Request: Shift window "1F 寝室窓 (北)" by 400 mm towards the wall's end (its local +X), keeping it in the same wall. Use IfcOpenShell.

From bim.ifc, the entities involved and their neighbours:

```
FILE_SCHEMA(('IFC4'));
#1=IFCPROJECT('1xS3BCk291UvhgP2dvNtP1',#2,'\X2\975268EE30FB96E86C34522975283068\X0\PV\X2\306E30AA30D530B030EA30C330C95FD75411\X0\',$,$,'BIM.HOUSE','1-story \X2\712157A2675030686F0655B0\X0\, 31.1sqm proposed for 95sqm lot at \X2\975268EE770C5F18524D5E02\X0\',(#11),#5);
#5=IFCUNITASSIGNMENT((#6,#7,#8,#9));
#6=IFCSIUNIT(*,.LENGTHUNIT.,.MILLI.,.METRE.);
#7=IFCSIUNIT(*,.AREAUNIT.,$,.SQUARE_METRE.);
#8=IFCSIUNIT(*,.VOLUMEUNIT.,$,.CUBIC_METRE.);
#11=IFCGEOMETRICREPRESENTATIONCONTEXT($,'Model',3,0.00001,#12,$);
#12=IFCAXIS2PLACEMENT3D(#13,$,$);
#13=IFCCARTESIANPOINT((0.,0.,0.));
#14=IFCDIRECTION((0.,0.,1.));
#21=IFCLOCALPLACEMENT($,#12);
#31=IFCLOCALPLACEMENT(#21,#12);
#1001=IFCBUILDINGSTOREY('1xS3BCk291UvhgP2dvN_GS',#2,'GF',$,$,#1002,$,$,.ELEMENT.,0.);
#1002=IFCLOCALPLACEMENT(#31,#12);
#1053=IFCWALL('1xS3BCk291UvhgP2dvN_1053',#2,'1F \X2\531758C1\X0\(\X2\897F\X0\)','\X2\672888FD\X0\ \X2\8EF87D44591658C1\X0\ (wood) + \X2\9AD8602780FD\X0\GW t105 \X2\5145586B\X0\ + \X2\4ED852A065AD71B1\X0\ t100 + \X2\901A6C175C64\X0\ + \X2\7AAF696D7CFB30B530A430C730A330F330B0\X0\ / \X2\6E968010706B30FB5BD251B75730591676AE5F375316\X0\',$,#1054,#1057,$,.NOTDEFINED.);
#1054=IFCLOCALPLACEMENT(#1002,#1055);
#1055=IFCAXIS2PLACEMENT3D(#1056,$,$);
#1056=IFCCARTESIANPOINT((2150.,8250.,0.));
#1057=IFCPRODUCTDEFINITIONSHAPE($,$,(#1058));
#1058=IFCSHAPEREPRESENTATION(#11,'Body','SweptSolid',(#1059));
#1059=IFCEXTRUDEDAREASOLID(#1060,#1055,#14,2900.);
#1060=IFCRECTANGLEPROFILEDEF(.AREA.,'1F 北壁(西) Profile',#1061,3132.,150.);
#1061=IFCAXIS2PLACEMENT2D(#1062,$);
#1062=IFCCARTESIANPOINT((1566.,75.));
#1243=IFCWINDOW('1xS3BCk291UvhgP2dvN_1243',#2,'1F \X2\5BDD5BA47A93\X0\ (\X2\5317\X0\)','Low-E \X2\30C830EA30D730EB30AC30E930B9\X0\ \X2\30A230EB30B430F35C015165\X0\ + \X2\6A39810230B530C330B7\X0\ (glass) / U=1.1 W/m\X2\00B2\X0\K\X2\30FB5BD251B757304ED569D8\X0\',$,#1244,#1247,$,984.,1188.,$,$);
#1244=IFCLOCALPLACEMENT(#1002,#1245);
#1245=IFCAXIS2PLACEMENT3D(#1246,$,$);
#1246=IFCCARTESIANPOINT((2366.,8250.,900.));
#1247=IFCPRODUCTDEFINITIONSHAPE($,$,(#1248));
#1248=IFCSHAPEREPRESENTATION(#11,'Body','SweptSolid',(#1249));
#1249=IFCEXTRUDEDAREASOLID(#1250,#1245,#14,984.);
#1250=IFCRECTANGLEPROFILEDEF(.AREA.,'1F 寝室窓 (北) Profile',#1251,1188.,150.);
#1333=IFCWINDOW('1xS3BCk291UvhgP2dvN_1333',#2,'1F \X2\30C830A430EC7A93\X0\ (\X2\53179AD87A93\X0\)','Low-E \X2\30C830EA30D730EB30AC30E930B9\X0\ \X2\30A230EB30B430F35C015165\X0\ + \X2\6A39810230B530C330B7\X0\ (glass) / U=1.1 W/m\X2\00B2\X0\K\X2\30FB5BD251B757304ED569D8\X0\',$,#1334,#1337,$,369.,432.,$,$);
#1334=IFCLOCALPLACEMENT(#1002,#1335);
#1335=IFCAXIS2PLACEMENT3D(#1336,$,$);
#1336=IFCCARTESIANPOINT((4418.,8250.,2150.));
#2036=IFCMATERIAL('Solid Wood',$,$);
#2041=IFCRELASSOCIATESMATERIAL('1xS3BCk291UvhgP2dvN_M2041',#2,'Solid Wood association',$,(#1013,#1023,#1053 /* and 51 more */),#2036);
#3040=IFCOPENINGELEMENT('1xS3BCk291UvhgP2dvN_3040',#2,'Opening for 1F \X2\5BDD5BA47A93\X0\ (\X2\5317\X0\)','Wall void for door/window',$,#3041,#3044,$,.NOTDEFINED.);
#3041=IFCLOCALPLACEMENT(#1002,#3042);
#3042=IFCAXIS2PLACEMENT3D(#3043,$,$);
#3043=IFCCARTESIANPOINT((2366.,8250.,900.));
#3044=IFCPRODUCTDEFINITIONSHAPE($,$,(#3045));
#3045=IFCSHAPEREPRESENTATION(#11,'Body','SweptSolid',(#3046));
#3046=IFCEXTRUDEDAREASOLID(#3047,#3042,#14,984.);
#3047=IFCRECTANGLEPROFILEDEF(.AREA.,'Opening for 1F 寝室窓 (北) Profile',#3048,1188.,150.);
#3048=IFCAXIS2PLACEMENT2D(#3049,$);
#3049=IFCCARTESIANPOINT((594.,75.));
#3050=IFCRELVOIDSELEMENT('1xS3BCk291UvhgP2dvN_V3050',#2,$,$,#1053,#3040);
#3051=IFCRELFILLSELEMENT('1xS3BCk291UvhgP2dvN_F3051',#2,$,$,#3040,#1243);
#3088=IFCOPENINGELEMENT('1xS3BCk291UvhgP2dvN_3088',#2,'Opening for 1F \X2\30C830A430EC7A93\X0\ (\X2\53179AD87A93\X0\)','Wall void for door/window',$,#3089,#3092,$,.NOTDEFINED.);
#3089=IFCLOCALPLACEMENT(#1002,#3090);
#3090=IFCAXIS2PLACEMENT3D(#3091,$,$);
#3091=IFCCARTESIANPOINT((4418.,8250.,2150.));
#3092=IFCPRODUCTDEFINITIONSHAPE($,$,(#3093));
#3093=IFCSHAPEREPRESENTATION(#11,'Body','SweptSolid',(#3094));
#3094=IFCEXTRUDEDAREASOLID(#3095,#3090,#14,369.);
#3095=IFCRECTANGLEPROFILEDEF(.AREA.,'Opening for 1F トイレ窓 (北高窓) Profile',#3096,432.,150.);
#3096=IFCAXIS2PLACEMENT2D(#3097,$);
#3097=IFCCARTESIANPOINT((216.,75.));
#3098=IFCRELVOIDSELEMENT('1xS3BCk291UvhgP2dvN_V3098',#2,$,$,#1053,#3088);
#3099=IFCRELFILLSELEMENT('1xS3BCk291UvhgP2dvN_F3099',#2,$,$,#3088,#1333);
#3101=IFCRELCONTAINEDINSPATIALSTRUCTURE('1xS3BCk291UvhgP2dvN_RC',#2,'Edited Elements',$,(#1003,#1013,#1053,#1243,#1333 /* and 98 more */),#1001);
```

```python
import ifcopenshell
import ifcopenshell.api.geometry
import ifcopenshell.util.placement
import ifcopenshell.util.unit

model = ifcopenshell.open("bim.ifc")
unit_scale = ifcopenshell.util.unit.calculate_unit_scale(model)

window = model.by_guid("1xS3BCk291UvhgP2dvN_1243")
opening = window.FillsVoids[0].RelatingOpeningElement
wall = opening.VoidsElements[0].RelatingBuildingElement

wall_matrix = ifcopenshell.util.placement.get_local_placement(wall.ObjectPlacement)
shift = wall_matrix[:3, 0] * 0.4 / unit_scale
before = ifcopenshell.util.placement.get_local_placement(window.ObjectPlacement)[:3, 3].copy()

# The window is not placed relative to its opening, so move both.
for product in (opening, window):
    matrix = ifcopenshell.util.placement.get_local_placement(product.ObjectPlacement)
    matrix[:3, 3] += shift
    ifcopenshell.api.geometry.edit_object_placement(model, product=product, matrix=matrix, is_si=False)

after = ifcopenshell.util.placement.get_local_placement(window.ObjectPlacement)[:3, 3]
print("window moved by", (after - before).round(3) + 0.0)

model.write("bim_edited.ifc")
```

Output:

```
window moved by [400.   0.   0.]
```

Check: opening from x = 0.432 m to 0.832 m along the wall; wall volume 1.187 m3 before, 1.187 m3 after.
